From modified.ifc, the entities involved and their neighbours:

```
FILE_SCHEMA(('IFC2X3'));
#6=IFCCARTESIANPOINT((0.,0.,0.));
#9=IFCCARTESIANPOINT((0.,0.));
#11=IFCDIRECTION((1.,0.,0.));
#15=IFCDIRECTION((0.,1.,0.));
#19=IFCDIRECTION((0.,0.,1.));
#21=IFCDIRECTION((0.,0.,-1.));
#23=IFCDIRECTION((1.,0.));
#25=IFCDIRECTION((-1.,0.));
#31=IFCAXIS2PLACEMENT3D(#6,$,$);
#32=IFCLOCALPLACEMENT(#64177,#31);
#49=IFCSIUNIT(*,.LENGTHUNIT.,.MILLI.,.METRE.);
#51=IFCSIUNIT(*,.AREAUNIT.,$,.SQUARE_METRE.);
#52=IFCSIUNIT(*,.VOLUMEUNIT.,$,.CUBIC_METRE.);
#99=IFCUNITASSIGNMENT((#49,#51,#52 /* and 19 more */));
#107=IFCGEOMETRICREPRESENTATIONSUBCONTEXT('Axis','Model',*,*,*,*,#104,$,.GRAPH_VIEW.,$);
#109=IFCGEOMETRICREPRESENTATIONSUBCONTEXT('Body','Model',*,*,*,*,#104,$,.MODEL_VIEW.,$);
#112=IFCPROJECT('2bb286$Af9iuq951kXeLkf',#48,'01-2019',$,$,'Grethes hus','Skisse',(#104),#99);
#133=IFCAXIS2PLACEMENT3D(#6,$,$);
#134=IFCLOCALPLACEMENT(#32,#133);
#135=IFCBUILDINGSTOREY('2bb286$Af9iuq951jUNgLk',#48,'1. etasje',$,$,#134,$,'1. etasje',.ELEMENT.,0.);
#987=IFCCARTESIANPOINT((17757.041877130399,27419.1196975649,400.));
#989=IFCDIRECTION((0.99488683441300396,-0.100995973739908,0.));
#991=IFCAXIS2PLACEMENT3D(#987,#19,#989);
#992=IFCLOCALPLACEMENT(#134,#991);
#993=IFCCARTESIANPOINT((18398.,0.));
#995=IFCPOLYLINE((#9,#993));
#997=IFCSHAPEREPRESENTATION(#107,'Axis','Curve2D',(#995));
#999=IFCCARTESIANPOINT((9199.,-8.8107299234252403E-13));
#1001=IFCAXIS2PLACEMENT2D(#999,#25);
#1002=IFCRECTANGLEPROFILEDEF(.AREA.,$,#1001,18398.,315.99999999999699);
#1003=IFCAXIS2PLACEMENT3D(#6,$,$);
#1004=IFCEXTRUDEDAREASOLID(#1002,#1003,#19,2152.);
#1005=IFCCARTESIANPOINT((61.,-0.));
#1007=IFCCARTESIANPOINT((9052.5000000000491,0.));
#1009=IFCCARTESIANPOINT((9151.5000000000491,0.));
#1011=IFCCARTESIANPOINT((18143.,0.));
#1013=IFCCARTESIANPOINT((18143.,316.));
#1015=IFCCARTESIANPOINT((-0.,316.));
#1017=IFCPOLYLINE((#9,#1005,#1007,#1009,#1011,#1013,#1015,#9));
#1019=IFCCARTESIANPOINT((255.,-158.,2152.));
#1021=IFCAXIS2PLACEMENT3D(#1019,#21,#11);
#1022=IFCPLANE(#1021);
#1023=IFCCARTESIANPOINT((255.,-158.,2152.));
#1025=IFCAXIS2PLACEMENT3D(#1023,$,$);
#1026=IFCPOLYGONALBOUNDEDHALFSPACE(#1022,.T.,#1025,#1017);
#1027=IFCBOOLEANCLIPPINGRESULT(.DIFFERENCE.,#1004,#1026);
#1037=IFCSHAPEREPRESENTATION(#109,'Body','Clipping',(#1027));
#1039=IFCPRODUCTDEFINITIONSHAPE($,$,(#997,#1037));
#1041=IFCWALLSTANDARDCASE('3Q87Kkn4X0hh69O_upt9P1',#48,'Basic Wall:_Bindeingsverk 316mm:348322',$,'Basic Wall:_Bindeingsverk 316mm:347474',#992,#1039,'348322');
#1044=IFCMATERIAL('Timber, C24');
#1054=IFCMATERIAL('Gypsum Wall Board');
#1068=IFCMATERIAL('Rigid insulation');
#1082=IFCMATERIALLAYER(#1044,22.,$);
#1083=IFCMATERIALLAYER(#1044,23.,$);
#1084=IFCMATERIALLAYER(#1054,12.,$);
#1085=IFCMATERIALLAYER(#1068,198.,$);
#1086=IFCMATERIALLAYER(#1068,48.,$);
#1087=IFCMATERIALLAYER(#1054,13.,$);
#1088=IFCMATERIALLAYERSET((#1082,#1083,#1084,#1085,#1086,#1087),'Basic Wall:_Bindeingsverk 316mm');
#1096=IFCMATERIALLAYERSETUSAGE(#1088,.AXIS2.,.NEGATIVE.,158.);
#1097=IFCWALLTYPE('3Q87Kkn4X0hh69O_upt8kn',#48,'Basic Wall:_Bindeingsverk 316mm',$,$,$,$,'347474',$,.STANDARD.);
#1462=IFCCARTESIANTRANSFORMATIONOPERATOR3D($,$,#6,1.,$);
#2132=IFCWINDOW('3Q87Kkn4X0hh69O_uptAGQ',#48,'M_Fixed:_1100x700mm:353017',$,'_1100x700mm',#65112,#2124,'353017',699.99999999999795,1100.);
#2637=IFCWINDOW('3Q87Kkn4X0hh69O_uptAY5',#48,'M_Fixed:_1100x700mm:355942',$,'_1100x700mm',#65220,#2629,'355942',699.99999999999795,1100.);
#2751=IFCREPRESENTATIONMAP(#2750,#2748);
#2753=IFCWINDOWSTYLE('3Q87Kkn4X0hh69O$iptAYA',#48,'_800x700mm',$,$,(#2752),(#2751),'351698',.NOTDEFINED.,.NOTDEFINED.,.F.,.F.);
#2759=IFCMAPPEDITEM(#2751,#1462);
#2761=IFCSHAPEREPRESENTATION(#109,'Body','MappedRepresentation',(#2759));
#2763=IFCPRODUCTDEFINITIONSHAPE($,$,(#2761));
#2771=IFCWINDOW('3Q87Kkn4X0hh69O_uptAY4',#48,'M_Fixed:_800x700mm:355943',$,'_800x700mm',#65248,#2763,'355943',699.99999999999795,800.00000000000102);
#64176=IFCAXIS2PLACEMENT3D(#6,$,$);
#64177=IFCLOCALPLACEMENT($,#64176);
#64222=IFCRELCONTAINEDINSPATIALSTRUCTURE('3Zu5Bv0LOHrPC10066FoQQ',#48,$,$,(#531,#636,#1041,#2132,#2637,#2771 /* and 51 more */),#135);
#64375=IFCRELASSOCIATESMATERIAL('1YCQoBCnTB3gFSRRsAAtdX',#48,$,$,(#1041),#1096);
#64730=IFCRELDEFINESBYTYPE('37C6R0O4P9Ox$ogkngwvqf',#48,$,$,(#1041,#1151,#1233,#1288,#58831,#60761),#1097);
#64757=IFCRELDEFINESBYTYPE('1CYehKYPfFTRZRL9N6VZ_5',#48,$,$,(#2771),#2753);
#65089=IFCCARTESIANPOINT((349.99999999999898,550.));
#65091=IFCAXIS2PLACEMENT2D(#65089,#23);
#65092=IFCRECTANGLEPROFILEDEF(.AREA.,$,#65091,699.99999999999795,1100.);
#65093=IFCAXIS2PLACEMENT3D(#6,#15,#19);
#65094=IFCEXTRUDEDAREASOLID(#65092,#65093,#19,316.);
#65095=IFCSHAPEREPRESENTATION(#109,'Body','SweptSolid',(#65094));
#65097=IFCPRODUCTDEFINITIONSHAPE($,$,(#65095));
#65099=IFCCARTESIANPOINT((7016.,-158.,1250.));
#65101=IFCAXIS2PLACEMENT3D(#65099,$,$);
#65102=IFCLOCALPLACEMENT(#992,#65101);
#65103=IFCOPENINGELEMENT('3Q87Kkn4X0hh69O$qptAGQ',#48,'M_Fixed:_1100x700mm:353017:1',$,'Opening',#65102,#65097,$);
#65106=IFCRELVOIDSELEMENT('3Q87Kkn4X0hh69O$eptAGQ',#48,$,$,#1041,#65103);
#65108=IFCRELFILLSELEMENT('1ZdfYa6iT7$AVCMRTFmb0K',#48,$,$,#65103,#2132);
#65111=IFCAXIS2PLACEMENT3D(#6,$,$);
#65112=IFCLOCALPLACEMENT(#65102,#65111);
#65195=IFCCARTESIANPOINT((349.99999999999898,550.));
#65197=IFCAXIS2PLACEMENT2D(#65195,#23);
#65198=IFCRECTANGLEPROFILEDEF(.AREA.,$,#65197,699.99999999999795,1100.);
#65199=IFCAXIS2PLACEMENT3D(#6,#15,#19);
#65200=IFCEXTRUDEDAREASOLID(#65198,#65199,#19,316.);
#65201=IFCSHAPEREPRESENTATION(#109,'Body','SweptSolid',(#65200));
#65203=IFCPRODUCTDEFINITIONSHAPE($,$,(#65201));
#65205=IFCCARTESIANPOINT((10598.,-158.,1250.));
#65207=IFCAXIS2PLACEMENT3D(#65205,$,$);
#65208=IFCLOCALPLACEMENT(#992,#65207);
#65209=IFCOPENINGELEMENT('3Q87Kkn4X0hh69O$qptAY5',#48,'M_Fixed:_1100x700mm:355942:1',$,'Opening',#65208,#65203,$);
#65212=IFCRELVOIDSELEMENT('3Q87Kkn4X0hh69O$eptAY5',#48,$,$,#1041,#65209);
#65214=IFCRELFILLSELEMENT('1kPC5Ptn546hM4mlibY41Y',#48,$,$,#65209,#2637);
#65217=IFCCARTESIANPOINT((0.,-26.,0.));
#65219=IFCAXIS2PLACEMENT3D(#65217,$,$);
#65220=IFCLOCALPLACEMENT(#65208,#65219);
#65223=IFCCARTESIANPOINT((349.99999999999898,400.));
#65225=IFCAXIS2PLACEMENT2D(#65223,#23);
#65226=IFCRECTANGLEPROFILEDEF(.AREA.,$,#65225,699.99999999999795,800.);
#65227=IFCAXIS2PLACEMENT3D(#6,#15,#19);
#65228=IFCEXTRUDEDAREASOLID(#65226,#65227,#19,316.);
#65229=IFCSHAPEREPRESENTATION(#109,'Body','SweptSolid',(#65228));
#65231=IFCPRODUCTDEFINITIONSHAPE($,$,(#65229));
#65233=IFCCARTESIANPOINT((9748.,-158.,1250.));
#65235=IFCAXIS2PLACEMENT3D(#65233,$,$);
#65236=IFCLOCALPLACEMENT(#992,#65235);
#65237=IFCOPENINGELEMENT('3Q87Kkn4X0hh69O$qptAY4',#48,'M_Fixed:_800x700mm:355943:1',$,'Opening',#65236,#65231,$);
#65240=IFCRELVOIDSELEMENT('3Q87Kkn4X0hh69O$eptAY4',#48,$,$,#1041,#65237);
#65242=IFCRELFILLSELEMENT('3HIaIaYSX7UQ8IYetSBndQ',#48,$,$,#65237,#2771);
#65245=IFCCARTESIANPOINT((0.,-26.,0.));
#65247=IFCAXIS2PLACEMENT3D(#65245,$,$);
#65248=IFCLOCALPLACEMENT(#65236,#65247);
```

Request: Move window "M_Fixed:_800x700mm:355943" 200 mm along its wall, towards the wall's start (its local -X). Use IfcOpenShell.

```python
import ifcopenshell
import ifcopenshell.api.geometry
import ifcopenshell.util.placement
import ifcopenshell.util.unit

model = ifcopenshell.open("modified.ifc")
unit_scale = ifcopenshell.util.unit.calculate_unit_scale(model)

window = model.by_guid("3Q87Kkn4X0hh69O_uptAY4")
opening = window.FillsVoids[0].RelatingOpeningElement
wall = opening.VoidsElements[0].RelatingBuildingElement

wall_matrix = ifcopenshell.util.placement.get_local_placement(wall.ObjectPlacement)
shift = wall_matrix[:3, 0] * -0.2 / unit_scale
before = ifcopenshell.util.placement.get_local_placement(window.ObjectPlacement)[:3, 3].copy()

# The window is placed relative to its opening, so it follows when the opening moves.
matrix = ifcopenshell.util.placement.get_local_placement(opening.ObjectPlacement)
matrix[:3, 3] += shift
ifcopenshell.api.geometry.edit_object_placement(
    model, product=opening, matrix=matrix, is_si=False, should_transform_children=True
)

after = ifcopenshell.util.placement.get_local_placement(window.ObjectPlacement)[:3, 3]
print("window moved by", (after - before).round(3) + 0.0)

model.write("modified_updated.ifc")
```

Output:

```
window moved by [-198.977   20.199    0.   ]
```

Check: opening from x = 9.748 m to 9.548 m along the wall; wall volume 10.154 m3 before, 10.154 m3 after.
